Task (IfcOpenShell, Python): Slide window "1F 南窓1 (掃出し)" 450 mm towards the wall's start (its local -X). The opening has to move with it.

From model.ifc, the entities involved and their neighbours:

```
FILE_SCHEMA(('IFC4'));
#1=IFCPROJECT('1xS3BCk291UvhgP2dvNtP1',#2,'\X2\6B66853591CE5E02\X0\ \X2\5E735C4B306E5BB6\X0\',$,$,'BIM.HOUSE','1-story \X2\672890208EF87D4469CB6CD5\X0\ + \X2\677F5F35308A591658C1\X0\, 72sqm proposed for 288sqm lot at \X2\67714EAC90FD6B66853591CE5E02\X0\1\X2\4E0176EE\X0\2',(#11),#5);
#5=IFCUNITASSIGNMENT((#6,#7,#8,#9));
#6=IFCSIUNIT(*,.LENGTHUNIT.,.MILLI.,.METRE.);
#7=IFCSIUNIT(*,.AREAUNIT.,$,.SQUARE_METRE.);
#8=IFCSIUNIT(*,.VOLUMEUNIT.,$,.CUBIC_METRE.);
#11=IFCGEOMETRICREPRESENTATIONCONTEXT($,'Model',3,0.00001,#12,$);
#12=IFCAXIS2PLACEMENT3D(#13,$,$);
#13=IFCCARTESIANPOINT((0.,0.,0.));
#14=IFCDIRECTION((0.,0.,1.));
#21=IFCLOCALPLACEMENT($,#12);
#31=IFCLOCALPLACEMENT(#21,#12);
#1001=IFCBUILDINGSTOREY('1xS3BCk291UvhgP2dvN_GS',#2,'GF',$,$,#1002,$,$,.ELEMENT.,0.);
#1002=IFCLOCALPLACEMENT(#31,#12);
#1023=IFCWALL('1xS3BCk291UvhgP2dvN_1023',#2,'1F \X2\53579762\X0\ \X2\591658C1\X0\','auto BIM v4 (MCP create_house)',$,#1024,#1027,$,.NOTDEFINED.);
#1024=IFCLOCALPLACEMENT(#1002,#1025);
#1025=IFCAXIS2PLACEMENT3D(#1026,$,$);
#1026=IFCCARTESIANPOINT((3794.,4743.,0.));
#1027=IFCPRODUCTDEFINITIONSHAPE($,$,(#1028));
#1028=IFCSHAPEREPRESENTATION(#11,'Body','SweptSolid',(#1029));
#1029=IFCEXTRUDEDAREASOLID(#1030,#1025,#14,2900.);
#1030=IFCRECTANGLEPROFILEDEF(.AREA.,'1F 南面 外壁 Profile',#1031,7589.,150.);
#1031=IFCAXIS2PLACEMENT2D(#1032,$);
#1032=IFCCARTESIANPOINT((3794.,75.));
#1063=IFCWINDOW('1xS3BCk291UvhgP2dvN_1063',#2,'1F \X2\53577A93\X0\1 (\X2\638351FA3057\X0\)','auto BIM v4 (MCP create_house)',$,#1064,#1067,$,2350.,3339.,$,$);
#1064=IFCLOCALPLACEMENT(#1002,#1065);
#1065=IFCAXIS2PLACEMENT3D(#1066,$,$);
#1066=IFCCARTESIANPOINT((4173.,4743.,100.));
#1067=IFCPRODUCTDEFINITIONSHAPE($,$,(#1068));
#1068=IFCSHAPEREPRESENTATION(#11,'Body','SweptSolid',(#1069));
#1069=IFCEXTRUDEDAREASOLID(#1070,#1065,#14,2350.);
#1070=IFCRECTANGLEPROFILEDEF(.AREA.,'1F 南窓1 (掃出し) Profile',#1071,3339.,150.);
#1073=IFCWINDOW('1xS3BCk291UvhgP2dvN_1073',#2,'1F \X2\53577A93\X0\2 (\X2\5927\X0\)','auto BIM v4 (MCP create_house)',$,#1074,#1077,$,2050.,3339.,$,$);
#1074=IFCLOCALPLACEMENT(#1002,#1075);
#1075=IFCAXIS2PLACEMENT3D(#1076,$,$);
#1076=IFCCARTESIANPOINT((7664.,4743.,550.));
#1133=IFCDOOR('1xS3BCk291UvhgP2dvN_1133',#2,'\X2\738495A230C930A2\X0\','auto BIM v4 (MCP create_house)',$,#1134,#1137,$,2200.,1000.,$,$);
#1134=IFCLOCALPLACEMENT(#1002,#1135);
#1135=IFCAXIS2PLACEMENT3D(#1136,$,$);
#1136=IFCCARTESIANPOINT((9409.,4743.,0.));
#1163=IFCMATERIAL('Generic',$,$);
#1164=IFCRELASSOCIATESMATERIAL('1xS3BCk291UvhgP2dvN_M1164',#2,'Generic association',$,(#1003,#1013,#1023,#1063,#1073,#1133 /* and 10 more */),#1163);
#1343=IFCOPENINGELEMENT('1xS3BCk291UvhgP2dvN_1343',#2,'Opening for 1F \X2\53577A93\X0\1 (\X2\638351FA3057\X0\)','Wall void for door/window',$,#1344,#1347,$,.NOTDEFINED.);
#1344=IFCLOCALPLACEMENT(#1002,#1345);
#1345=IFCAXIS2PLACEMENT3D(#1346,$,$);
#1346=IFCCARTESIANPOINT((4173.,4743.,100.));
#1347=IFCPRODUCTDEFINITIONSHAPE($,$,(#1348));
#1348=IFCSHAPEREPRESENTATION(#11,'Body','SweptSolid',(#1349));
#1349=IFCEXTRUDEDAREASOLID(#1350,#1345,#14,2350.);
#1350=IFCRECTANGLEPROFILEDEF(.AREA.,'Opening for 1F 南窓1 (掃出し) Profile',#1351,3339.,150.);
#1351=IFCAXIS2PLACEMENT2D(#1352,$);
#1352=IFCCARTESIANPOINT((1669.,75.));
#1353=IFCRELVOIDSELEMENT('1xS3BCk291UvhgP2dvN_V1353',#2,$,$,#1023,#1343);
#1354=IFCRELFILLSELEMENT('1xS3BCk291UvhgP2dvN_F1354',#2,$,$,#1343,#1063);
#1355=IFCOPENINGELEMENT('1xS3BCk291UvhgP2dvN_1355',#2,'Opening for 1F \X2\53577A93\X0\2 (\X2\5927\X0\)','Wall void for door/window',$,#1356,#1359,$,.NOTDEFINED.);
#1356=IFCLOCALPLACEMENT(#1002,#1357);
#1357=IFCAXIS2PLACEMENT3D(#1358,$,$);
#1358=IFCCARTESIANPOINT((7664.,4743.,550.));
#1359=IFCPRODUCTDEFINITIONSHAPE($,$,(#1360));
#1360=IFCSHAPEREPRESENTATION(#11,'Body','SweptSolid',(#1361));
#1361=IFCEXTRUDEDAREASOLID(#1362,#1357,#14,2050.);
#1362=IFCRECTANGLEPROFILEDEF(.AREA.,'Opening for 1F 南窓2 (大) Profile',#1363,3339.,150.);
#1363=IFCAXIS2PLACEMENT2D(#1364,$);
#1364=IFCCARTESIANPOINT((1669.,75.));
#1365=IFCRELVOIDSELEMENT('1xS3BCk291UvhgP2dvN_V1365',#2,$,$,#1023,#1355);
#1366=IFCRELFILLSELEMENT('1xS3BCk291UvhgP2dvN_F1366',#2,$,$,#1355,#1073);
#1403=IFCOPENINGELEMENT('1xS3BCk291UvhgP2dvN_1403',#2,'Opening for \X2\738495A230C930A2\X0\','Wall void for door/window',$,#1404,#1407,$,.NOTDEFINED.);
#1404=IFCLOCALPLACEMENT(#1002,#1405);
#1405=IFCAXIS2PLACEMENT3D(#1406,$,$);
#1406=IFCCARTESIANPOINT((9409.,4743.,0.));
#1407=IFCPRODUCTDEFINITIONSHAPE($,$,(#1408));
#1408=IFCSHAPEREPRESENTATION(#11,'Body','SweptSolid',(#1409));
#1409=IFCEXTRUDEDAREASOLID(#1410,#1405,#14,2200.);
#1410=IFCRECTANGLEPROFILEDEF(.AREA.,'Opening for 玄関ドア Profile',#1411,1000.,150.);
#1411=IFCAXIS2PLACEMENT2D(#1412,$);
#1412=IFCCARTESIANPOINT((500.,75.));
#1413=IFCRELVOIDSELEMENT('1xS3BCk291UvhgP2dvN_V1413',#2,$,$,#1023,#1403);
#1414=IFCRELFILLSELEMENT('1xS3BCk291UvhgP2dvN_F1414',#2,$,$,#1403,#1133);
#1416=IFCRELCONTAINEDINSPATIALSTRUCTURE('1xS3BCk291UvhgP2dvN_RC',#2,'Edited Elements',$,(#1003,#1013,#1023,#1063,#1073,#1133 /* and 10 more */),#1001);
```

```python
import ifcopenshell
import ifcopenshell.api.geometry
import ifcopenshell.util.placement

model = ifcopenshell.open("model.ifc")

window = model.by_guid("1xS3BCk291UvhgP2dvN_1063")
opening = window.FillsVoids[0].RelatingOpeningElement
wall = opening.VoidsElements[0].RelatingBuildingElement

wall_matrix = ifcopenshell.util.placement.get_local_placement(wall.ObjectPlacement)
shift = wall_matrix[:3, 0] * -450.0
before = ifcopenshell.util.placement.get_local_placement(window.ObjectPlacement)[:3, 3].copy()

# The window is not placed relative to its opening, so move both.
for product in (opening, window):
    matrix = ifcopenshell.util.placement.get_local_placement(product.ObjectPlacement)
    matrix[:3, 3] += shift
    ifcopenshell.api.geometry.edit_object_placement(model, product=product, matrix=matrix, is_si=False)

after = ifcopenshell.util.placement.get_local_placement(window.ObjectPlacement)[:3, 3]
print("window moved by", (after - before).round(3) + 0.0)

model.write("model_rev.ifc")
```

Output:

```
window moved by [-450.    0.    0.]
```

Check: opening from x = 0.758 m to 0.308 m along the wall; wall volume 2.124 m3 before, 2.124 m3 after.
